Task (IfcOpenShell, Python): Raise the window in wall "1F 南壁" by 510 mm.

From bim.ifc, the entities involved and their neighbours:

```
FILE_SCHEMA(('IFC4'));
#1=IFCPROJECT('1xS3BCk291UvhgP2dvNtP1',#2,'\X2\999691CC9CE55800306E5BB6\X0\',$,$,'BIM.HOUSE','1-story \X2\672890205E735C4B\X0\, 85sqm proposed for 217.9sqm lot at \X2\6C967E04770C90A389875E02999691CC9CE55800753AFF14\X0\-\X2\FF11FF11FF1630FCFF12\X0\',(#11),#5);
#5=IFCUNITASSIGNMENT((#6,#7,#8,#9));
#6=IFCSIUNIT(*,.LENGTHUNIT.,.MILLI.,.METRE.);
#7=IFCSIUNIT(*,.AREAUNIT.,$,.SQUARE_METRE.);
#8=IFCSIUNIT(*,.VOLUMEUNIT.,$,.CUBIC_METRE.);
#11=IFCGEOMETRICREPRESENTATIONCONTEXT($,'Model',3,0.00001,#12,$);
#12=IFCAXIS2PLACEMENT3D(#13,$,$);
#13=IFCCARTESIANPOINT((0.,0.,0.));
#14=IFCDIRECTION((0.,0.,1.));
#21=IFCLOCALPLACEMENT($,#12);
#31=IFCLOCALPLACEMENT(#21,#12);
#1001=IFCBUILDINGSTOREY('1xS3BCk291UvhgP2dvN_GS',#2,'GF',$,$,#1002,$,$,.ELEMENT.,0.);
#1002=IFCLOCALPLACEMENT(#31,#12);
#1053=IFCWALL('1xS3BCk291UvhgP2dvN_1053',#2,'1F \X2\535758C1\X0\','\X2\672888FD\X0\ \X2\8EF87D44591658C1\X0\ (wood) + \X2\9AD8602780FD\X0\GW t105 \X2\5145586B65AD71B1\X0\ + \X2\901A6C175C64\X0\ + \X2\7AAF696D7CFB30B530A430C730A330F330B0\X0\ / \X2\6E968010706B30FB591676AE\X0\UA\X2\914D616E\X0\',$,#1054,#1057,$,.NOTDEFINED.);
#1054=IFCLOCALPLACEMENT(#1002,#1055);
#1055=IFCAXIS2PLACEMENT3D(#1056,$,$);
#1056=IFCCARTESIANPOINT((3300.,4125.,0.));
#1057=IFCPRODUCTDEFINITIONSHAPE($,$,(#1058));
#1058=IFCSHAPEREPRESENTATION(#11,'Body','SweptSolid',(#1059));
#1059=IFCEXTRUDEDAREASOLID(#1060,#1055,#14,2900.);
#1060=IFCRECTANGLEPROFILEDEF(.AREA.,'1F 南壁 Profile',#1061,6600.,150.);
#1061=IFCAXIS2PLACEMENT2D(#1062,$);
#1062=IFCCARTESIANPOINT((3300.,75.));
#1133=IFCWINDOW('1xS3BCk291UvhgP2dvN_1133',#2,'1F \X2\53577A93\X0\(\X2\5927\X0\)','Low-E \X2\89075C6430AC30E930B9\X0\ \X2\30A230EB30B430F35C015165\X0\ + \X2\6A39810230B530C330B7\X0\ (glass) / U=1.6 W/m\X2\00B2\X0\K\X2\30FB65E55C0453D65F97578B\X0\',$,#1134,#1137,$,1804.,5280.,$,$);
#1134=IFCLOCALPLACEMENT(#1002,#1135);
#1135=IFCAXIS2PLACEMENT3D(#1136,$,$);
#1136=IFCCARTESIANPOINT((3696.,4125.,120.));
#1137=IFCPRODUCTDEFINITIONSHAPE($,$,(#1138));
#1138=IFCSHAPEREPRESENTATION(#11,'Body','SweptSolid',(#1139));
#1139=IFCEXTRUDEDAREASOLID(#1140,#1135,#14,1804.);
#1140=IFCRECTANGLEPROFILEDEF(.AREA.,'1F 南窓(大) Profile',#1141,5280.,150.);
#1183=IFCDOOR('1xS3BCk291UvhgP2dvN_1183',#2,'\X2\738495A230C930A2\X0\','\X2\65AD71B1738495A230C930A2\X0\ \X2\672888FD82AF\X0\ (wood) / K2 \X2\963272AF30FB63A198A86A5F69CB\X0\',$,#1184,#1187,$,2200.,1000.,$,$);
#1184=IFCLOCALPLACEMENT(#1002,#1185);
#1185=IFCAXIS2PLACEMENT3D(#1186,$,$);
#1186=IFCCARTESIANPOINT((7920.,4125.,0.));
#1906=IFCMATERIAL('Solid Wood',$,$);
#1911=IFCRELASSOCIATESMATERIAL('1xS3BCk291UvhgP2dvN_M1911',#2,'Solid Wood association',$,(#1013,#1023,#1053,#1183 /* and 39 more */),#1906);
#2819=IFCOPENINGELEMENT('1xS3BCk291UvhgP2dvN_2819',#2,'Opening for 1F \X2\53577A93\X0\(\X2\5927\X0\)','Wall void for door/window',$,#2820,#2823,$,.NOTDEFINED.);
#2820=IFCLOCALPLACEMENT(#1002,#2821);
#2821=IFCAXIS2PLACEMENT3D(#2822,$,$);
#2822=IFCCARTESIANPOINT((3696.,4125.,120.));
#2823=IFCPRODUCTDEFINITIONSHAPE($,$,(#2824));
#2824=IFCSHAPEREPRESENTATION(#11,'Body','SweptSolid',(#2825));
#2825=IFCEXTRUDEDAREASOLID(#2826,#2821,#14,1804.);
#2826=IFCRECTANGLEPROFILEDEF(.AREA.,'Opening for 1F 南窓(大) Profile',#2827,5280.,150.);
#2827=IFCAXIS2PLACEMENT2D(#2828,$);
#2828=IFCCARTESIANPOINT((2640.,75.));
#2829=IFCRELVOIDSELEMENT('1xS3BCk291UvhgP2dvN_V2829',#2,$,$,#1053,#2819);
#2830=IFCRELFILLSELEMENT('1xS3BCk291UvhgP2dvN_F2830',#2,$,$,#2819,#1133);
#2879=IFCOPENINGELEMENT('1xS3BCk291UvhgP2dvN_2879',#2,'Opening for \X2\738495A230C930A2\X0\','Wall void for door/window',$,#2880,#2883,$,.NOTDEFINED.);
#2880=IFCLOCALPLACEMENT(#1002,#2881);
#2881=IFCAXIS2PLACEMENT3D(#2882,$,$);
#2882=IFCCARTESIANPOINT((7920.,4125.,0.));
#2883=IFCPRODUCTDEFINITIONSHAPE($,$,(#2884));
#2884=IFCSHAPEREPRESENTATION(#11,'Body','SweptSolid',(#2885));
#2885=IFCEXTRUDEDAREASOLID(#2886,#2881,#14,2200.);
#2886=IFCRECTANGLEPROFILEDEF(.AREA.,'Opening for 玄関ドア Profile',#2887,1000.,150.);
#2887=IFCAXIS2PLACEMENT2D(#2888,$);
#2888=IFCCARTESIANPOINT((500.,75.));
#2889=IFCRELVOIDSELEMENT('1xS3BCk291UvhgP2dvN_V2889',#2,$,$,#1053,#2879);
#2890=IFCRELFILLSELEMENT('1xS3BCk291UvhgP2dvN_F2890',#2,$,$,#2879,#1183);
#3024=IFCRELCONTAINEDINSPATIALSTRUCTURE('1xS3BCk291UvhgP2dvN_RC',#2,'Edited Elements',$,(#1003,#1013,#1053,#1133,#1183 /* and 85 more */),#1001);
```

```python
import numpy as np
import ifcopenshell
import ifcopenshell.api.geometry
import ifcopenshell.util.placement
import ifcopenshell.util.unit

model = ifcopenshell.open("bim.ifc")
unit_scale = ifcopenshell.util.unit.calculate_unit_scale(model)

window = model.by_guid("1xS3BCk291UvhgP2dvN_1133")
opening = window.FillsVoids[0].RelatingOpeningElement
dz = 0.51 / unit_scale

shift = np.array([0.0, 0.0, dz])
# The window is not placed relative to its opening, so move both.
for product in (opening, window):
    matrix = ifcopenshell.util.placement.get_local_placement(product.ObjectPlacement)
    matrix[:3, 3] += shift
    ifcopenshell.api.geometry.edit_object_placement(model, product=product, matrix=matrix, is_si=False)

print(f"moved by {dz * unit_scale:+.3f} m")

model.write("bim_edited.ifc")
```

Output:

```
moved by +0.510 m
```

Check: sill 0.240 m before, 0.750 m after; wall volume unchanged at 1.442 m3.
